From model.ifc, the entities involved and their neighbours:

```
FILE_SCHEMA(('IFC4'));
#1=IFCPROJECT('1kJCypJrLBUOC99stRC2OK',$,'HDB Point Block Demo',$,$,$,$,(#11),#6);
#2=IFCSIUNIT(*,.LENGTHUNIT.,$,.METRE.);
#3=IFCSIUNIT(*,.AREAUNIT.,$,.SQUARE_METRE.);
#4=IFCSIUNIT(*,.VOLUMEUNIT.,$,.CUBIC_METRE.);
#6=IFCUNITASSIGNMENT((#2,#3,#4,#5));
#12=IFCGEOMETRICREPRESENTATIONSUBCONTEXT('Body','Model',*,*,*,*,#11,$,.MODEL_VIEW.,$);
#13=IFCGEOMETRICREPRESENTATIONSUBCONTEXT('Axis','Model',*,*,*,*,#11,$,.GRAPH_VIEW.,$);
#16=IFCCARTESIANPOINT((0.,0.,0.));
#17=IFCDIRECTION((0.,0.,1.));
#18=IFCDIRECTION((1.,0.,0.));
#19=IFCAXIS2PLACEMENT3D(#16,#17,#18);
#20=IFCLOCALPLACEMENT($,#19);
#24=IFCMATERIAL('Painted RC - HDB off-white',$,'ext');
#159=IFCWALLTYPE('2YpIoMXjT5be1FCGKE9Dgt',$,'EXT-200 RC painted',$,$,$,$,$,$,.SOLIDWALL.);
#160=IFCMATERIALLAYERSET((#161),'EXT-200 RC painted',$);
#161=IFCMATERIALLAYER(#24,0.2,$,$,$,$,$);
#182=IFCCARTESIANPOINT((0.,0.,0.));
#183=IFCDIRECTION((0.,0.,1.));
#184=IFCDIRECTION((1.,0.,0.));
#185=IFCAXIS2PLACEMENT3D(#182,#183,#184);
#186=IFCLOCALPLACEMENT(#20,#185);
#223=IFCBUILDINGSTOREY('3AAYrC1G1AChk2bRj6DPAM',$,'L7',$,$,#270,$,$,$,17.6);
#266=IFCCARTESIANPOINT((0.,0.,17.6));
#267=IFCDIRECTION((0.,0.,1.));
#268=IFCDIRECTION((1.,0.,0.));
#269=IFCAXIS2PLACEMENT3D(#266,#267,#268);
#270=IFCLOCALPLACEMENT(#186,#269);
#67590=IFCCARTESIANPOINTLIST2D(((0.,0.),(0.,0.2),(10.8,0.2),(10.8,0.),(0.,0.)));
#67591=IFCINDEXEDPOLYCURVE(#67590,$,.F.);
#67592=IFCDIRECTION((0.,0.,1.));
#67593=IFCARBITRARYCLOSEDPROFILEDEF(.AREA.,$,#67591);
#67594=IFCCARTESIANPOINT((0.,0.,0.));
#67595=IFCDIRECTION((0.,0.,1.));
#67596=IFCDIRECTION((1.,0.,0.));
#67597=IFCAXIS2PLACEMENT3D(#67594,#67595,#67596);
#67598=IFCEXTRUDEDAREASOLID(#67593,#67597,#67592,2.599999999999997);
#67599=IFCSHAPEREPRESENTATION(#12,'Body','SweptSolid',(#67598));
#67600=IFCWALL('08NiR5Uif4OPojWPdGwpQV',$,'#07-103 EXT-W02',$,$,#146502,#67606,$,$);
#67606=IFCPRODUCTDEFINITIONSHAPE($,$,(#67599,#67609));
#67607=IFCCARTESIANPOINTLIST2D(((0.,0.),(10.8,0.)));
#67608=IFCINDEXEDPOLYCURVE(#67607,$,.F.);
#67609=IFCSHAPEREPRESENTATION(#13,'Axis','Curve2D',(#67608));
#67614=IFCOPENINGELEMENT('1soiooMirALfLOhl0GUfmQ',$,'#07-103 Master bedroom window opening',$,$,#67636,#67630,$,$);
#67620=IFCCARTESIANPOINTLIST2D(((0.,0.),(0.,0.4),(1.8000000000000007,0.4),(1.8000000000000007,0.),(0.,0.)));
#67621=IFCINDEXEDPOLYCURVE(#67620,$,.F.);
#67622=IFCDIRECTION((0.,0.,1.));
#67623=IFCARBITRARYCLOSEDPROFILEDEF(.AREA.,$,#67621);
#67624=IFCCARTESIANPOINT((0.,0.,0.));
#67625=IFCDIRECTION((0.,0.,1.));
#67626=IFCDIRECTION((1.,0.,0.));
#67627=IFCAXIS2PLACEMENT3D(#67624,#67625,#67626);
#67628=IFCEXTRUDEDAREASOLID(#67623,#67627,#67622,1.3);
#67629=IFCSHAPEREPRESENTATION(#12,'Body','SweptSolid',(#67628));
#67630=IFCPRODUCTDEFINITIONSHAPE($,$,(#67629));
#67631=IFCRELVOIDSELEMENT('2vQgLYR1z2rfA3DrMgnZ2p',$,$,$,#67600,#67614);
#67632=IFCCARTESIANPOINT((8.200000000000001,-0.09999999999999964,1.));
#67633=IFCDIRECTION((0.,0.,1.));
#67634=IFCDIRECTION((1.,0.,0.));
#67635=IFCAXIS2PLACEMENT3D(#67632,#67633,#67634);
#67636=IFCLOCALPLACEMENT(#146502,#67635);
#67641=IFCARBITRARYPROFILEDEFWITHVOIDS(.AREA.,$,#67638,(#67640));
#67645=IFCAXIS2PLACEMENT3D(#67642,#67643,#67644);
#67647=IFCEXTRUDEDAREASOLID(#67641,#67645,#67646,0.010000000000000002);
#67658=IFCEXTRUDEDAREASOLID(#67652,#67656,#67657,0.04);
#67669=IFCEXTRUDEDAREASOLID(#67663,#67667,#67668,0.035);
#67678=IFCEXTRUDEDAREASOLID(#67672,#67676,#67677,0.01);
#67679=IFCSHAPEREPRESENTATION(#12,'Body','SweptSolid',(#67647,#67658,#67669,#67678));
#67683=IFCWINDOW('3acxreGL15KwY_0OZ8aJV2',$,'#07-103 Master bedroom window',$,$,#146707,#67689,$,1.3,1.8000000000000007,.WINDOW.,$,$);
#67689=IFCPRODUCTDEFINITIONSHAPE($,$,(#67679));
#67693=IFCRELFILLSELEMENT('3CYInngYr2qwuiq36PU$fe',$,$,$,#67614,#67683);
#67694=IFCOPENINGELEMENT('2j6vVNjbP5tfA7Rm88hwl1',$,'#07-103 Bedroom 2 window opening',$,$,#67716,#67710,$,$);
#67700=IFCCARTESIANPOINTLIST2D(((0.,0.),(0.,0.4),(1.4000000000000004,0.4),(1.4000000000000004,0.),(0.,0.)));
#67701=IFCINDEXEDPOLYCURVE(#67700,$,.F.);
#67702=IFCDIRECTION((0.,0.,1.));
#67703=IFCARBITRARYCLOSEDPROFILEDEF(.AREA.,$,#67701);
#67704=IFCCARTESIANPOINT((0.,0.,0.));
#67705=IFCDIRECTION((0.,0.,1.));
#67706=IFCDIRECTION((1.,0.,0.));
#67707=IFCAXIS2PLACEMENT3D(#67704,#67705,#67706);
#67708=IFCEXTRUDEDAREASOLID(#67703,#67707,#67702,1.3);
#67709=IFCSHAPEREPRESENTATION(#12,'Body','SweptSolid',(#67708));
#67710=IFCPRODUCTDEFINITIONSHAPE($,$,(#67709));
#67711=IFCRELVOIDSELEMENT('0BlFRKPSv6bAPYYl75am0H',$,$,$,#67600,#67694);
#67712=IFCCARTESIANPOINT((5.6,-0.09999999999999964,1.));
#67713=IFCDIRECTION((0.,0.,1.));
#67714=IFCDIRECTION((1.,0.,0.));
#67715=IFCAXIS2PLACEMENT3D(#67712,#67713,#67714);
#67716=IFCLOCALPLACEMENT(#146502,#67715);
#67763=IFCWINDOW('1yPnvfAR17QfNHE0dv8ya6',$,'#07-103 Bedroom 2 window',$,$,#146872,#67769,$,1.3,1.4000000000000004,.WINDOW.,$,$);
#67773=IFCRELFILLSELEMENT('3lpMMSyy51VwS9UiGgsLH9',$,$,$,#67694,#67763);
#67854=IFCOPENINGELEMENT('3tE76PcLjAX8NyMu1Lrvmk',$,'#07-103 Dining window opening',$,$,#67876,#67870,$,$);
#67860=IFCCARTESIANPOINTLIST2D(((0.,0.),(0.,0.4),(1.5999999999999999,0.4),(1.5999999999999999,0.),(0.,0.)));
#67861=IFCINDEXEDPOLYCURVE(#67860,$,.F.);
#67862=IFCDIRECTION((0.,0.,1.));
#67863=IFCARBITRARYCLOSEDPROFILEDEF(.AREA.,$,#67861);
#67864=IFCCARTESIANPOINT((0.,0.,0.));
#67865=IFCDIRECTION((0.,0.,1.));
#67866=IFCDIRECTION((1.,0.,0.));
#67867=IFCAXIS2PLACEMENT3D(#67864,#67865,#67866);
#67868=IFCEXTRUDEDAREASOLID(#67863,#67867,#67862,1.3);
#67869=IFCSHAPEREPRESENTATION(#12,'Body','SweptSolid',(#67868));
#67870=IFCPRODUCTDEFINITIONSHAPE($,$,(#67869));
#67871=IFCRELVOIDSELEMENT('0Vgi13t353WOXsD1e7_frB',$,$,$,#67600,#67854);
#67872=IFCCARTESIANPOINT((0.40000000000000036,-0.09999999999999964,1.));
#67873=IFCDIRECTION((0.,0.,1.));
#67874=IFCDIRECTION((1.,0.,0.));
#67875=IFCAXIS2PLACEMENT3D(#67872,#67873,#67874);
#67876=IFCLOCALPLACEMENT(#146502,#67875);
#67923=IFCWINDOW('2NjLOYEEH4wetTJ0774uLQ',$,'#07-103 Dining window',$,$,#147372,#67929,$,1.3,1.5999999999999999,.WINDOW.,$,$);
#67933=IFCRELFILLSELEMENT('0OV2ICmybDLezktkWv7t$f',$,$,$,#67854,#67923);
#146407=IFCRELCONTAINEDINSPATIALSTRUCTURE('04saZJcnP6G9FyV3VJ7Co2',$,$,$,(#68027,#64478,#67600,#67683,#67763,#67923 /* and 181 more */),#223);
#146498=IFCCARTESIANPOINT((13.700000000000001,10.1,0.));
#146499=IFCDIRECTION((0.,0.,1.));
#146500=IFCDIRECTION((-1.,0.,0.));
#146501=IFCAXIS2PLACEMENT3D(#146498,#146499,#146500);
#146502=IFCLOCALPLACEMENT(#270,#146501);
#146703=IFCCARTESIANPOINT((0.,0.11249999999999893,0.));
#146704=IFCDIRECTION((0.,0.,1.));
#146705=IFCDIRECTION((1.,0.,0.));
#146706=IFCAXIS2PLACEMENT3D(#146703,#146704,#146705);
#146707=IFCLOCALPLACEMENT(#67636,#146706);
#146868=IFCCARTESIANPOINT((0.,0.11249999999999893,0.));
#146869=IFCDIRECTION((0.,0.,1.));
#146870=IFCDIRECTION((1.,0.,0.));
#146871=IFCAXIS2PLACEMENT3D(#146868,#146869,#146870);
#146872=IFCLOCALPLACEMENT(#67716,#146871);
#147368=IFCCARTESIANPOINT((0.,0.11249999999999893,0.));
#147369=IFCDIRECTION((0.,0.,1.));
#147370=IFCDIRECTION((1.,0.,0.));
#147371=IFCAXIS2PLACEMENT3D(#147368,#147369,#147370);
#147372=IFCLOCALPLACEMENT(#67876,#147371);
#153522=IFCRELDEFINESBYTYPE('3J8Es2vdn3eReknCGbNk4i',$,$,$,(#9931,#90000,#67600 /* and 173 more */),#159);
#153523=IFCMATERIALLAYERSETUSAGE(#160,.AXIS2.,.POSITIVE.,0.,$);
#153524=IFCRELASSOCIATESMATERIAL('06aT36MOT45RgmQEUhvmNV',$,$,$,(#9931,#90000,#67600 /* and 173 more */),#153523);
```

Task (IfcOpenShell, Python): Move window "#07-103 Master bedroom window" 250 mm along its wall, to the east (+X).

```python
import ifcopenshell
import ifcopenshell.api.geometry
import ifcopenshell.util.placement
import ifcopenshell.util.unit

model = ifcopenshell.open("model.ifc")
unit_scale = ifcopenshell.util.unit.calculate_unit_scale(model)

window = model.by_guid("3acxreGL15KwY_0OZ8aJV2")
opening = window.FillsVoids[0].RelatingOpeningElement
wall = opening.VoidsElements[0].RelatingBuildingElement

wall_matrix = ifcopenshell.util.placement.get_local_placement(wall.ObjectPlacement)
shift = wall_matrix[:3, 0] * -0.25 / unit_scale
before = ifcopenshell.util.placement.get_local_placement(window.ObjectPlacement)[:3, 3].copy()

# The window is placed relative to its opening, so it follows when the opening moves.
matrix = ifcopenshell.util.placement.get_local_placement(opening.ObjectPlacement)
matrix[:3, 3] += shift
ifcopenshell.api.geometry.edit_object_placement(
    model, product=opening, matrix=matrix, is_si=False, should_transform_children=True
)

after = ifcopenshell.util.placement.get_local_placement(window.ObjectPlacement)[:3, 3]
print("window moved by", (after - before).round(3) + 0.0)

model.write("model-out.ifc")
```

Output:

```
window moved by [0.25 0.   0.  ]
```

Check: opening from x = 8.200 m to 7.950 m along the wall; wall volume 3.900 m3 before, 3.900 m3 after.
